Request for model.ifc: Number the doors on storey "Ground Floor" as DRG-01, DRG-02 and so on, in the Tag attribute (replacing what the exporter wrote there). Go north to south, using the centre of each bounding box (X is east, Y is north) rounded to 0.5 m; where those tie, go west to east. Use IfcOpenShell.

First a look at what the model holds.

```python
import ifcopenshell
import ifcopenshell.util.element
import ifcopenshell.util.placement

model = ifcopenshell.open("model.ifc")
print(model.schema)
storey = next(s for s in model.by_type("IfcBuildingStorey") if s.Name == "Ground Floor")
doors = [e for e in ifcopenshell.util.element.get_decomposition(storey) if e.is_a("IfcDoor")]
for e in sorted(doors, key=lambda e: e.id()):
    origin = ifcopenshell.util.placement.get_local_placement(e.ObjectPlacement)[:3, 3]
    print(e.id(), e.Tag, e.Name, origin.round(2) + 0.0, sep=" | ")
```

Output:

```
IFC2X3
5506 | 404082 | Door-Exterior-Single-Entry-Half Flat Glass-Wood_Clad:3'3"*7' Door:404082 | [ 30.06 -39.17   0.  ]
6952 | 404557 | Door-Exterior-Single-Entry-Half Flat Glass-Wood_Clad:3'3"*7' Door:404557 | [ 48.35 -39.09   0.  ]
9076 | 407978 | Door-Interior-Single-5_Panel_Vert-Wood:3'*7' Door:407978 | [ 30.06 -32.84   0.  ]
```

```python
import ifcopenshell
import ifcopenshell.geom
import ifcopenshell.util.element
import ifcopenshell.util.shape

model = ifcopenshell.open("model.ifc")
settings = ifcopenshell.geom.settings()
settings.set("use-world-coords", True)


def centre(element):
    shape = ifcopenshell.geom.create_shape(settings, element)
    return ifcopenshell.util.shape.get_bbox_centroid(shape.geometry)


storey = next(s for s in model.by_type("IfcBuildingStorey") if s.Name == "Ground Floor")
doors = [e for e in ifcopenshell.util.element.get_decomposition(storey) if e.is_a("IfcDoor")]

# Insertion points can sit at a corner or the storey origin, so sort by the geometry (in metres).
centres = {e: centre(e) for e in doors}
doors.sort(key=lambda e: (-round(centres[e][1] / 0.5), centres[e][0]))

for i, e in enumerate(doors, start=1):
    number = f"DRG-{i:02d}"
    e.Tag = number
    print(e.id(), number)

model.write("model_updated.ifc")
```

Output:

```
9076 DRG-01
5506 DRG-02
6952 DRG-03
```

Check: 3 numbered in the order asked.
